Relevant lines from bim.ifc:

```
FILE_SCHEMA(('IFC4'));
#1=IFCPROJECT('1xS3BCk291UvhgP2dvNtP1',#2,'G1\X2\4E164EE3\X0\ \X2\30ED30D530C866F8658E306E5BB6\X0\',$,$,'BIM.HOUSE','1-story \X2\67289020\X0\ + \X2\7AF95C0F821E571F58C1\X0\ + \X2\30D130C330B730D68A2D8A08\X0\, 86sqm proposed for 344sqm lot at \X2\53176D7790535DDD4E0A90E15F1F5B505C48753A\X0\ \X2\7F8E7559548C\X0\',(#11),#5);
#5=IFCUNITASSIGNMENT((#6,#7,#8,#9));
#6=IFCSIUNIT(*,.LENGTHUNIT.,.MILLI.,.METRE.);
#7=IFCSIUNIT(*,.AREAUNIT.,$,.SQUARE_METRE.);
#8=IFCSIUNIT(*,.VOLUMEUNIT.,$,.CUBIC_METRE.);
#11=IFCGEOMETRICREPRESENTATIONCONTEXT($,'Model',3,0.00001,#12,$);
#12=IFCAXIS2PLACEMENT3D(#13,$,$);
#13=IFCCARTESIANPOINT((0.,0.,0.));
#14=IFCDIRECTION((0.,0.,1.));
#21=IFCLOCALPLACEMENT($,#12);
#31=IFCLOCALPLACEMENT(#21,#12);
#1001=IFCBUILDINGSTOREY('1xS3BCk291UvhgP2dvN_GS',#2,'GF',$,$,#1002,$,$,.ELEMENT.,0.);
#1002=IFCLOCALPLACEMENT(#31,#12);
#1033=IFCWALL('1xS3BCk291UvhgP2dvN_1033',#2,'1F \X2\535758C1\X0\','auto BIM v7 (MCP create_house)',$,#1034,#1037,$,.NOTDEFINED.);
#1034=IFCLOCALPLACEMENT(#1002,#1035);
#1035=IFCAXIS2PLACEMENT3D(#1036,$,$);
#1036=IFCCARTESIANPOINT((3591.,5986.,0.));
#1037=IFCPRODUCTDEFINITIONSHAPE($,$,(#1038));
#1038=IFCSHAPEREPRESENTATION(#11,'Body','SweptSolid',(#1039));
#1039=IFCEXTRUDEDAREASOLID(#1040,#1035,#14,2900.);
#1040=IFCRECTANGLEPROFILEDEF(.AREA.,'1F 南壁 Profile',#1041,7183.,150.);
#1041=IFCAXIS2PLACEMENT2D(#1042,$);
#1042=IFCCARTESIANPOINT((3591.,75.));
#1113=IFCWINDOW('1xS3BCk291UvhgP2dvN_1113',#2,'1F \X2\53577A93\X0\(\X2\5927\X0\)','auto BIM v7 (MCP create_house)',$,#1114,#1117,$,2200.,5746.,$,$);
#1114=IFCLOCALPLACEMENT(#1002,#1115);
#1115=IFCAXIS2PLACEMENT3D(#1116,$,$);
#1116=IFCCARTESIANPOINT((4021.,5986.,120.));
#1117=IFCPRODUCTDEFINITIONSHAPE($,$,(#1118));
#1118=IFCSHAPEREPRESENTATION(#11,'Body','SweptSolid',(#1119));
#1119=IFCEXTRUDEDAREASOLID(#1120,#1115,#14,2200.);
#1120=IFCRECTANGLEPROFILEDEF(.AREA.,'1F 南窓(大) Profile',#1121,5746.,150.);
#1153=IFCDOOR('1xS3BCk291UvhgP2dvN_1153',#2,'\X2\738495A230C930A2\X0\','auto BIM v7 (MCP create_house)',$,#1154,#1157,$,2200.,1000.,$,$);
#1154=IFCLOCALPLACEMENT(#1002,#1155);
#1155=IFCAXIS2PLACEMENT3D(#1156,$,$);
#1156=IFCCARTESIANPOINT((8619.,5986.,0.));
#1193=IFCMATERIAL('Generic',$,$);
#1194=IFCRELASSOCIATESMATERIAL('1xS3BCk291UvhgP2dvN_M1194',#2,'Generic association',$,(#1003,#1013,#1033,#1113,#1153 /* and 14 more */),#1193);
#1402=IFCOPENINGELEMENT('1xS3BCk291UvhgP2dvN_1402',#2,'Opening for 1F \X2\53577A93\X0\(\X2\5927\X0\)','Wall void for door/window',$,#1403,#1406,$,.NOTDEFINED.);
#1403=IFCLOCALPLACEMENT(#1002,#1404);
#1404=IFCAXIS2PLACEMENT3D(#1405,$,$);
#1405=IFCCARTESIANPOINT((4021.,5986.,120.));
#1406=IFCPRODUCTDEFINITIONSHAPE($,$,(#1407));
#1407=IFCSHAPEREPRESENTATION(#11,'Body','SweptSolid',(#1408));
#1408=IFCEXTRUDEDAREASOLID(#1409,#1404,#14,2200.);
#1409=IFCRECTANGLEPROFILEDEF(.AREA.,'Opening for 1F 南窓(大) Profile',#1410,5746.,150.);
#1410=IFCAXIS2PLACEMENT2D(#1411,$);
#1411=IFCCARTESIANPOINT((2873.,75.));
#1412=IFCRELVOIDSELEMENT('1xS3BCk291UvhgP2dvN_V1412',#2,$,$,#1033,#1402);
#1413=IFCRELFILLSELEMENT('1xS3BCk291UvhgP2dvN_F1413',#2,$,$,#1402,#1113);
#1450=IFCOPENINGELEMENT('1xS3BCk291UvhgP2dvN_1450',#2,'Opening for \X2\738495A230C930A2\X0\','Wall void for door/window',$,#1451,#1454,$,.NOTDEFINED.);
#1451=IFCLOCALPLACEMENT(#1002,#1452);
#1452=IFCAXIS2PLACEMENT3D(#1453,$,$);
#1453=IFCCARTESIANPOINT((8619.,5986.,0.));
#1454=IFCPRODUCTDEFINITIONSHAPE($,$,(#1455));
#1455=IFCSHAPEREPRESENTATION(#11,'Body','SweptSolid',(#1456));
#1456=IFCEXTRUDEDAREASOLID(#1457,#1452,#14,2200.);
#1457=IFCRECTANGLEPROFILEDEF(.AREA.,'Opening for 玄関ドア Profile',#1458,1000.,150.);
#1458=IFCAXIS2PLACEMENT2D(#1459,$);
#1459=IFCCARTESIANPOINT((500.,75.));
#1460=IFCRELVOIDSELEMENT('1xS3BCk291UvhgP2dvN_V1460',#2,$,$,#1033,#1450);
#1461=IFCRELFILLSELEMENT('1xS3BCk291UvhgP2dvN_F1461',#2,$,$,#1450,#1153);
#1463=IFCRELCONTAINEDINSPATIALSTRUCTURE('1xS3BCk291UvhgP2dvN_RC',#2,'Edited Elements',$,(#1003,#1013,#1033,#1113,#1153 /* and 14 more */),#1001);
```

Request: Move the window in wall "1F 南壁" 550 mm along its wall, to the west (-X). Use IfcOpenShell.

```python
import ifcopenshell
import ifcopenshell.api.geometry
import ifcopenshell.util.placement
import ifcopenshell.util.unit

model = ifcopenshell.open("bim.ifc")
unit_scale = ifcopenshell.util.unit.calculate_unit_scale(model)

window = model.by_guid("1xS3BCk291UvhgP2dvN_1113")
opening = window.FillsVoids[0].RelatingOpeningElement
wall = opening.VoidsElements[0].RelatingBuildingElement

wall_matrix = ifcopenshell.util.placement.get_local_placement(wall.ObjectPlacement)
shift = wall_matrix[:3, 0] * -0.55 / unit_scale
before = ifcopenshell.util.placement.get_local_placement(window.ObjectPlacement)[:3, 3].copy()

# The window is not placed relative to its opening, so move both.
for product in (opening, window):
    matrix = ifcopenshell.util.placement.get_local_placement(product.ObjectPlacement)
    matrix[:3, 3] += shift
    ifcopenshell.api.geometry.edit_object_placement(model, product=product, matrix=matrix, is_si=False)

after = ifcopenshell.util.placement.get_local_placement(window.ObjectPlacement)[:3, 3]
print("window moved by", (after - before).round(3) + 0.0)

model.write("bim_v2.ifc")
```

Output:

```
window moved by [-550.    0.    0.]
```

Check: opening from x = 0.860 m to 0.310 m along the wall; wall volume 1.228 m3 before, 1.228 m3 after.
